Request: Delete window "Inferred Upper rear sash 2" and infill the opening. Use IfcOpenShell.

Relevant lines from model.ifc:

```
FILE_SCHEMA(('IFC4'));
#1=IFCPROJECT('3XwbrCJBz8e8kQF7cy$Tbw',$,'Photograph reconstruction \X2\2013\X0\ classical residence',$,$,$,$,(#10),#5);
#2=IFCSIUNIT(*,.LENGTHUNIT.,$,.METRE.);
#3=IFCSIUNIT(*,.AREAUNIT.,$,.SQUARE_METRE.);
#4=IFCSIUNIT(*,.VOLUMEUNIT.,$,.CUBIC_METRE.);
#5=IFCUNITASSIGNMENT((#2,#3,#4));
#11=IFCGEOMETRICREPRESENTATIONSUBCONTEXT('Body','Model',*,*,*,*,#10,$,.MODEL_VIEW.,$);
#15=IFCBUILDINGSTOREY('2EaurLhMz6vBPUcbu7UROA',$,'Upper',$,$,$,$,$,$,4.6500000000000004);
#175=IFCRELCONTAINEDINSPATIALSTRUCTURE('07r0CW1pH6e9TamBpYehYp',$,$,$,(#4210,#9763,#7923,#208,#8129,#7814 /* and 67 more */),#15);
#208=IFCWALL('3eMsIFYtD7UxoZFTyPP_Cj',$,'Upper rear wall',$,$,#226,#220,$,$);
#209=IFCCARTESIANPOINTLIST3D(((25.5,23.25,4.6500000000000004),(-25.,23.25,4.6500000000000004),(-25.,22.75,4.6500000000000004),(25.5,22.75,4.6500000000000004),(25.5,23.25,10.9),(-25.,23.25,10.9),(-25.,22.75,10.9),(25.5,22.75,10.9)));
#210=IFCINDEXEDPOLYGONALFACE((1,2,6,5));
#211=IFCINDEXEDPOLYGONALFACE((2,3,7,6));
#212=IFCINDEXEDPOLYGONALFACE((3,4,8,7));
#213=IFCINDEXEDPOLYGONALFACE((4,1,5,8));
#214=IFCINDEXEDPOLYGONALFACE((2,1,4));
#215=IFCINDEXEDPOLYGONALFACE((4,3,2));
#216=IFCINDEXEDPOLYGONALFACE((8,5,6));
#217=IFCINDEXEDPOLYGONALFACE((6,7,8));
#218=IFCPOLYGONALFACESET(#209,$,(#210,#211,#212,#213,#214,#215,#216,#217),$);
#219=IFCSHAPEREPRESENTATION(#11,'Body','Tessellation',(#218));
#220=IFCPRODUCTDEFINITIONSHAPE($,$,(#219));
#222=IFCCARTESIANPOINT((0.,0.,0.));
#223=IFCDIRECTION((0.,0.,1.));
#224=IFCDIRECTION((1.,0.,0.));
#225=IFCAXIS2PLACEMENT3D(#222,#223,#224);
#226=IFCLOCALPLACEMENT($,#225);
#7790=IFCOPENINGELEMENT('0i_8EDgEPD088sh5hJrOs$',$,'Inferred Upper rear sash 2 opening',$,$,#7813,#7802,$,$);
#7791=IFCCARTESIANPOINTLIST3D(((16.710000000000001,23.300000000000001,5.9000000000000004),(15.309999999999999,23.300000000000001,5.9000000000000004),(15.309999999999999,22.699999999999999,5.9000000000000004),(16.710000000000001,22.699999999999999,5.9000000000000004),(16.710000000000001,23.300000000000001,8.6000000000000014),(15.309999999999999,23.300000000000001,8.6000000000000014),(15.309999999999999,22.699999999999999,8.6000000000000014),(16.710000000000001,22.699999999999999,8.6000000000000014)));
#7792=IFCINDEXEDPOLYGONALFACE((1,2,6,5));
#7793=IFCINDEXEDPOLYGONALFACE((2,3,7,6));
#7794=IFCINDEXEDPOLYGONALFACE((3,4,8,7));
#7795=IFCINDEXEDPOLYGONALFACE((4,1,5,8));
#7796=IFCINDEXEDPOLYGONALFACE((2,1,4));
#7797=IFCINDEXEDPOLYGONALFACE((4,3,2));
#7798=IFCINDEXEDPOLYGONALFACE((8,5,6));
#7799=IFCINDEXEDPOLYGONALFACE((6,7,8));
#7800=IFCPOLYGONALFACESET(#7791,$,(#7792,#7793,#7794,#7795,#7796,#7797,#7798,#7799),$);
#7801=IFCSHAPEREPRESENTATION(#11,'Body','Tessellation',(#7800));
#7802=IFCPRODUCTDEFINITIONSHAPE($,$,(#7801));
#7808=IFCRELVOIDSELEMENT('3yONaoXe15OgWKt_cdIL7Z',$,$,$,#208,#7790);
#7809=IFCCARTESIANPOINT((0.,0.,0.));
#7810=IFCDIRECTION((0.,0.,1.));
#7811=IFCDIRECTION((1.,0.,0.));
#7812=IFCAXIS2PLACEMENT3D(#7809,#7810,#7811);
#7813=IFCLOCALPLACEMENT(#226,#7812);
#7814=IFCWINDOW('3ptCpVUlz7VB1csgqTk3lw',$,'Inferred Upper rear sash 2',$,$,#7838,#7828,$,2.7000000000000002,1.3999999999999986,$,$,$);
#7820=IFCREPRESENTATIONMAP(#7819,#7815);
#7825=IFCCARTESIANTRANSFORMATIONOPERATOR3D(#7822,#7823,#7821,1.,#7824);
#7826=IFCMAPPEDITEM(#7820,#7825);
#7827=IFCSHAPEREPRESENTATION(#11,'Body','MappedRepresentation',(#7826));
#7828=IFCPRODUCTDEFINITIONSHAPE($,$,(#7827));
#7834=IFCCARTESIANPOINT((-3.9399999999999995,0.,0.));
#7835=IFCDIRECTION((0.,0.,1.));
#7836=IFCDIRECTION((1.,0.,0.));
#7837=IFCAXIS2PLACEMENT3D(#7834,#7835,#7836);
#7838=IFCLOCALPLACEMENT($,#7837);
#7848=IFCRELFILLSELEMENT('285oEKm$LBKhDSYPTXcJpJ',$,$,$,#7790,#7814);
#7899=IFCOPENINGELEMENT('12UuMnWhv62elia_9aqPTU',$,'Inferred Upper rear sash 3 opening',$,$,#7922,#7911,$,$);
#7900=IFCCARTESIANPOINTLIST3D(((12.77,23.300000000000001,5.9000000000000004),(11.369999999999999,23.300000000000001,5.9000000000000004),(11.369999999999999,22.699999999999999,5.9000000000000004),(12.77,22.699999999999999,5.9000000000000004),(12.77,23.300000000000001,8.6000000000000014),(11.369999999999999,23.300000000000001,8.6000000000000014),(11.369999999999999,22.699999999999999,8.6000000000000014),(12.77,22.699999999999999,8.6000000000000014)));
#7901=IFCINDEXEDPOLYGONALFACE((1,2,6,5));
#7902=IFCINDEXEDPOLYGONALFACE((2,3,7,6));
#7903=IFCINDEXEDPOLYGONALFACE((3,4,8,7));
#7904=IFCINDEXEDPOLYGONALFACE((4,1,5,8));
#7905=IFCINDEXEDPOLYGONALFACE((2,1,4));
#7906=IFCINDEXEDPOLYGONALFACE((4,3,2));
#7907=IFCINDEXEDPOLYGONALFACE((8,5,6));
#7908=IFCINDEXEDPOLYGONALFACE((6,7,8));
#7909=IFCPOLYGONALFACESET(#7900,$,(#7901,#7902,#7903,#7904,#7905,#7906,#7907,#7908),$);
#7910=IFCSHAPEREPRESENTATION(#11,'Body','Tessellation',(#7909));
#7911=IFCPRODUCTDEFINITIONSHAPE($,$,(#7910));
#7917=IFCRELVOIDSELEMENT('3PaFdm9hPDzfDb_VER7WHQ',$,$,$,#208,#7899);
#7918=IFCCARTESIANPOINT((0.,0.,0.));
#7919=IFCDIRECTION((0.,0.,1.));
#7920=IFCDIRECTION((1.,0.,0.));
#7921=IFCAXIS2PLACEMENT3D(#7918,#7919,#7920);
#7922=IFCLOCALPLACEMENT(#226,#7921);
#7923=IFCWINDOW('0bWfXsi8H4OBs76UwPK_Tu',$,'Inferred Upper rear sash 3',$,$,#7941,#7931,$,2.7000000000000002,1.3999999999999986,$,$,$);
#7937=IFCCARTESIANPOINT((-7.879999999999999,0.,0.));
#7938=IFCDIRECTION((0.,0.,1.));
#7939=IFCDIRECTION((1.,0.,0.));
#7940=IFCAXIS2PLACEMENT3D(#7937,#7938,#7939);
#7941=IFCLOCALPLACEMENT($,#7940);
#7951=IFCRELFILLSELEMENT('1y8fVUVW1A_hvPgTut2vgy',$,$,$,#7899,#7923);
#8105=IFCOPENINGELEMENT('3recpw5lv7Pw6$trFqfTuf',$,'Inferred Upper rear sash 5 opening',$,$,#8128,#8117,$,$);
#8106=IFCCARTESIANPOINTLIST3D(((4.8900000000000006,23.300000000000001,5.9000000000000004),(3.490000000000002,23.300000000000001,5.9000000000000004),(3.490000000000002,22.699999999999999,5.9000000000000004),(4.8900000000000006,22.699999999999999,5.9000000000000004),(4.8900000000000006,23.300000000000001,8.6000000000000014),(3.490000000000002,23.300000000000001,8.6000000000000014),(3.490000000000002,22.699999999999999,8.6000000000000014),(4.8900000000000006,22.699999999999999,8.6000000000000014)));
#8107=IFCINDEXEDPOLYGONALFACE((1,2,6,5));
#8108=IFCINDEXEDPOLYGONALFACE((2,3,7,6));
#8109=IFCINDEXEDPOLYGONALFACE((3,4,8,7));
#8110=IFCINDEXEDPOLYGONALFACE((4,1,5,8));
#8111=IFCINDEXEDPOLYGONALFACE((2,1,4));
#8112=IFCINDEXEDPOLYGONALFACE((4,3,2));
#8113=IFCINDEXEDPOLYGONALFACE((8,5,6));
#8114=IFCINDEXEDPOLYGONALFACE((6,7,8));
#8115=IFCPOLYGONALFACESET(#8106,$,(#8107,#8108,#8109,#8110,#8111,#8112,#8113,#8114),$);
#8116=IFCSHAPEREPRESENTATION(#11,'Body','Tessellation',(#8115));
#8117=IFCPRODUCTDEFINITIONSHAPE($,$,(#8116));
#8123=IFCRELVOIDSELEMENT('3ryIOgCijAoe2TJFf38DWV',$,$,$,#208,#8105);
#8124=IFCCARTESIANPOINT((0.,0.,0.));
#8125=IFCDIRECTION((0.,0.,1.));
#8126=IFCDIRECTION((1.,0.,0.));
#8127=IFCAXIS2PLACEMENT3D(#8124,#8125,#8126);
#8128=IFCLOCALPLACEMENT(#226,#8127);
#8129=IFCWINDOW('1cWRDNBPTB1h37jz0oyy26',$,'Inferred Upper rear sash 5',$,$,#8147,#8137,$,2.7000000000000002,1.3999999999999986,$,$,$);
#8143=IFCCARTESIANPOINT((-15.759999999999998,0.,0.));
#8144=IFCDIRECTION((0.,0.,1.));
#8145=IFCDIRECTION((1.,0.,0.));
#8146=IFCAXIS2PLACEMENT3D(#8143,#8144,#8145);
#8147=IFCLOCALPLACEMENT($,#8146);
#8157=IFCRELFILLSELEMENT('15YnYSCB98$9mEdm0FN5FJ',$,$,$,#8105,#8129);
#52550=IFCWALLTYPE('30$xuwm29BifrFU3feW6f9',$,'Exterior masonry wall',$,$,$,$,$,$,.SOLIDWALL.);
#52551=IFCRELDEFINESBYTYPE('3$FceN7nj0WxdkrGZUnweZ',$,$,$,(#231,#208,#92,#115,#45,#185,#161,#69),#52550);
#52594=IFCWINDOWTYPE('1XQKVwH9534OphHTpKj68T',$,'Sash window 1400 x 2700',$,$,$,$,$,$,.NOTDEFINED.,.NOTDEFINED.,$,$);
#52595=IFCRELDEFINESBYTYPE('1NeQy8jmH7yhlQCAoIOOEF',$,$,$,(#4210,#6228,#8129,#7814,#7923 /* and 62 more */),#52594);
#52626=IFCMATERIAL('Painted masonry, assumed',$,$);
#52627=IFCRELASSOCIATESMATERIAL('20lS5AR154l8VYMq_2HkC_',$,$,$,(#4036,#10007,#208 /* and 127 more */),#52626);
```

```python
import ifcopenshell
import ifcopenshell.api.feature
import ifcopenshell.api.root
import ifcopenshell.geom
import ifcopenshell.util.shape

model = ifcopenshell.open("model.ifc")
settings = ifcopenshell.geom.settings()


def volume(element):
    """Net volume in cubic metres, openings subtracted."""
    shape = ifcopenshell.geom.create_shape(settings, element)
    return ifcopenshell.util.shape.get_volume(shape.geometry)


window = model.by_guid("3ptCpVUlz7VB1csgqTk3lw")
opening = window.FillsVoids[0].RelatingOpeningElement
wall = opening.VoidsElements[0].RelatingBuildingElement
before = volume(wall)

ifcopenshell.api.root.remove_product(model, product=window)
ifcopenshell.api.feature.remove_feature(model, feature=opening)

after = volume(wall)

print(f"wall volume {before:.3f} -> {after:.3f} m3")

model.write("model_rev.ifc")
```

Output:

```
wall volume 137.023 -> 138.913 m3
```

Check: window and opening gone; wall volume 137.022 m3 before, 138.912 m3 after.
